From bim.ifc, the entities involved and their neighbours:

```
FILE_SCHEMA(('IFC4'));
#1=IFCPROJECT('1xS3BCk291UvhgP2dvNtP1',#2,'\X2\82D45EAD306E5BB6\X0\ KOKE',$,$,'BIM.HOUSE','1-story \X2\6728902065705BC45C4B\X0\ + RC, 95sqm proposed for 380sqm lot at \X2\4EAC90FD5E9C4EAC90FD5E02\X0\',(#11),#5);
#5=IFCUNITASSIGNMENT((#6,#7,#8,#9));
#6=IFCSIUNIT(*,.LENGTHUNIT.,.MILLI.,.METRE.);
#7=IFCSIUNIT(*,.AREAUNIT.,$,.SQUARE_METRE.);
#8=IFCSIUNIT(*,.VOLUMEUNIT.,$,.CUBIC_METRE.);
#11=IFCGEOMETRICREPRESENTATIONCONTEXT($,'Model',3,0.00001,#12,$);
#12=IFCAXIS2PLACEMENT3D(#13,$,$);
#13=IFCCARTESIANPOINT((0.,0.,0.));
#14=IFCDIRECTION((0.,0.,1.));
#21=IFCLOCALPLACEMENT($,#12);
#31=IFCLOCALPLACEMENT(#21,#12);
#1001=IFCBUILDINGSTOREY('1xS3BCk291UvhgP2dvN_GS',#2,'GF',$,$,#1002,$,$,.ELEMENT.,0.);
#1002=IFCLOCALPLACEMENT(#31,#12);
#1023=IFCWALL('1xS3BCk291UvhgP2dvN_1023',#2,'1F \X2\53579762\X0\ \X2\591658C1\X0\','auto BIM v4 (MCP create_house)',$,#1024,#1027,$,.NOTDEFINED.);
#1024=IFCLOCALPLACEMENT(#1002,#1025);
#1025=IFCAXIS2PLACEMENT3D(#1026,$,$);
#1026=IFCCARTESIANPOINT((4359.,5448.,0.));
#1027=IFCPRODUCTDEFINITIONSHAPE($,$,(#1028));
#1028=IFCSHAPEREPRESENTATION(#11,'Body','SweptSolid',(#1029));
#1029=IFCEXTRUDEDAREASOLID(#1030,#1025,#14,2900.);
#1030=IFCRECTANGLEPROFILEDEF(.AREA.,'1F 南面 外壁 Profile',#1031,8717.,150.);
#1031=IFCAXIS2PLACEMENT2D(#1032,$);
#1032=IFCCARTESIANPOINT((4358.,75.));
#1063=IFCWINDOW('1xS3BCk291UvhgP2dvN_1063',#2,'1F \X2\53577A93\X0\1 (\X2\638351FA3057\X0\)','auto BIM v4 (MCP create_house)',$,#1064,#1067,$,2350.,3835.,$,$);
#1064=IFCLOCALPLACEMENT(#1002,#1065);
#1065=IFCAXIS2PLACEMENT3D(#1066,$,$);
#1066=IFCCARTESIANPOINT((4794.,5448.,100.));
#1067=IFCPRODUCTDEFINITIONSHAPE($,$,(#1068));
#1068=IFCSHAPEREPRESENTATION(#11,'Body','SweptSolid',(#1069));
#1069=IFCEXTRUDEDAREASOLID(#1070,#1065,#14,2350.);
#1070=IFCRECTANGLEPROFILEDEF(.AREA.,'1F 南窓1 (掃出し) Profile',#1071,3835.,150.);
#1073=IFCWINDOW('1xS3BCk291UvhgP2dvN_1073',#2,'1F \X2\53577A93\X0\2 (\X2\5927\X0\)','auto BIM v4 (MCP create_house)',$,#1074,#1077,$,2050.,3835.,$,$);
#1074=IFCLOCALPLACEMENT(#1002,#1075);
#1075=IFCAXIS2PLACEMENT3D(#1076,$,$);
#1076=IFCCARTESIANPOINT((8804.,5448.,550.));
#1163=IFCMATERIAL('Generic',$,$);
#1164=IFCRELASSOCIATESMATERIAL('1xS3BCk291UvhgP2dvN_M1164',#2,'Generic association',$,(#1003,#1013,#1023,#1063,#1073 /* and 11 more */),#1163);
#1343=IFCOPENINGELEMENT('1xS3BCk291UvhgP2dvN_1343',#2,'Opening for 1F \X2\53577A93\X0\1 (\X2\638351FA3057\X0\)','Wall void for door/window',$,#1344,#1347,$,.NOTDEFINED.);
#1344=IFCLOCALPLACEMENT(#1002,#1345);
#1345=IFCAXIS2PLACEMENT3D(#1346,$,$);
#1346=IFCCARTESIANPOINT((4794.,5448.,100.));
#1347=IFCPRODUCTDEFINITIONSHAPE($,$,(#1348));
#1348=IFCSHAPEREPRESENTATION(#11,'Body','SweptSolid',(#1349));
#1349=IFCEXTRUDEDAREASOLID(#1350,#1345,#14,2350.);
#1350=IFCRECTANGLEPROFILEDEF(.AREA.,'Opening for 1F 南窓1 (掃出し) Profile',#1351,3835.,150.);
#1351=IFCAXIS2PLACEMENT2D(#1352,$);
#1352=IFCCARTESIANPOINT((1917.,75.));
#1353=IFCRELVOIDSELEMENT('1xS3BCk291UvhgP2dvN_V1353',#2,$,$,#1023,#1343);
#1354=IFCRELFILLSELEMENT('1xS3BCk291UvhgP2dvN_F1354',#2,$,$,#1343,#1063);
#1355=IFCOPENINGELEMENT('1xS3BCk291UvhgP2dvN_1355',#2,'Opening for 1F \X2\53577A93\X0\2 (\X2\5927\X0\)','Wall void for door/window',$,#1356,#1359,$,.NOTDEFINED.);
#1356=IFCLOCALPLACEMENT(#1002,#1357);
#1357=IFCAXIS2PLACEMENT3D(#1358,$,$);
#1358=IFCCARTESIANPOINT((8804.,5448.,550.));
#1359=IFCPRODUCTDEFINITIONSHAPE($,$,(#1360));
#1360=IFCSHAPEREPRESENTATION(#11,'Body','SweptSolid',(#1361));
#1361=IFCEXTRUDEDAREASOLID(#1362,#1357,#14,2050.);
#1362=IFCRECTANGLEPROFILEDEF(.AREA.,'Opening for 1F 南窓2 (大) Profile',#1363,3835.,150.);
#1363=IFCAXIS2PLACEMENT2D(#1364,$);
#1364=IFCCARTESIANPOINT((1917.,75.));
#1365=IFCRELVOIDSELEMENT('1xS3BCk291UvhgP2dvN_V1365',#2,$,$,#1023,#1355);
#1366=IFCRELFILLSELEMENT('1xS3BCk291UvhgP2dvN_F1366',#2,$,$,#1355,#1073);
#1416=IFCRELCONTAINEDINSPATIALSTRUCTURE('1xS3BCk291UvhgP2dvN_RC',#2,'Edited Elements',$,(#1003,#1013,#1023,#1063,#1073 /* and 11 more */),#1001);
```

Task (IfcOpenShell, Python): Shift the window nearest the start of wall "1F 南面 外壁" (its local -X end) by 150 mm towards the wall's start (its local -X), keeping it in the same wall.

```python
import ifcopenshell
import ifcopenshell.api.geometry
import ifcopenshell.util.placement

model = ifcopenshell.open("bim.ifc")

window = model.by_guid("1xS3BCk291UvhgP2dvN_1063")
opening = window.FillsVoids[0].RelatingOpeningElement
wall = opening.VoidsElements[0].RelatingBuildingElement

wall_matrix = ifcopenshell.util.placement.get_local_placement(wall.ObjectPlacement)
shift = wall_matrix[:3, 0] * -150.0
before = ifcopenshell.util.placement.get_local_placement(window.ObjectPlacement)[:3, 3].copy()

# The window is not placed relative to its opening, so move both.
for product in (opening, window):
    matrix = ifcopenshell.util.placement.get_local_placement(product.ObjectPlacement)
    matrix[:3, 3] += shift
    ifcopenshell.api.geometry.edit_object_placement(model, product=product, matrix=matrix, is_si=False)

after = ifcopenshell.util.placement.get_local_placement(window.ObjectPlacement)[:3, 3]
print("window moved by", (after - before).round(3) + 0.0)

model.write("bim_v2.ifc")
```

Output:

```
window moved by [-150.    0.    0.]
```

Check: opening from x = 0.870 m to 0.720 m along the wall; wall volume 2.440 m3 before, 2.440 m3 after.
